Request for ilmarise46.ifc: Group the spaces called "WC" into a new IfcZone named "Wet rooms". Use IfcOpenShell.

First a look at what the model holds.

```python
import ifcopenshell

model = ifcopenshell.open("ilmarise46.ifc")
print(model.schema)
seen = {}
for space in model.by_type("IfcSpace"):
    seen[space.LongName] = seen.get(space.LongName, 0) + 1
for name, count in sorted(seen.items(), key=str):
    print(count, "x", name)
print("zones:", [z.Name for z in model.by_type("IfcZone")][:20])
```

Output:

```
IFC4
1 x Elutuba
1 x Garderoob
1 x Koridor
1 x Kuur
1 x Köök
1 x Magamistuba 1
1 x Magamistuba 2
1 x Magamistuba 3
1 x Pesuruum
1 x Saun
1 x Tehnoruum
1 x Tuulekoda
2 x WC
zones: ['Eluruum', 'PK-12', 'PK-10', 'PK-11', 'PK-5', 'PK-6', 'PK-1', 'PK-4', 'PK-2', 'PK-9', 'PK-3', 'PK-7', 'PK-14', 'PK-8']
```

```python
import ifcopenshell
import ifcopenshell.api.group
import ifcopenshell.api.root

model = ifcopenshell.open("ilmarise46.ifc")

names = {"WC"}
spaces = [s for s in model.by_type("IfcSpace") if s.LongName in names]

zone = ifcopenshell.api.root.create_entity(model, ifc_class="IfcZone", name="Wet rooms")
ifcopenshell.api.group.assign_group(model, products=spaces, group=zone)
print(len(spaces), "spaces in", zone.Name)

model.write("ilmarise46_v2.ifc")
```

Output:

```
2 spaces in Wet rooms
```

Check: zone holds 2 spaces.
